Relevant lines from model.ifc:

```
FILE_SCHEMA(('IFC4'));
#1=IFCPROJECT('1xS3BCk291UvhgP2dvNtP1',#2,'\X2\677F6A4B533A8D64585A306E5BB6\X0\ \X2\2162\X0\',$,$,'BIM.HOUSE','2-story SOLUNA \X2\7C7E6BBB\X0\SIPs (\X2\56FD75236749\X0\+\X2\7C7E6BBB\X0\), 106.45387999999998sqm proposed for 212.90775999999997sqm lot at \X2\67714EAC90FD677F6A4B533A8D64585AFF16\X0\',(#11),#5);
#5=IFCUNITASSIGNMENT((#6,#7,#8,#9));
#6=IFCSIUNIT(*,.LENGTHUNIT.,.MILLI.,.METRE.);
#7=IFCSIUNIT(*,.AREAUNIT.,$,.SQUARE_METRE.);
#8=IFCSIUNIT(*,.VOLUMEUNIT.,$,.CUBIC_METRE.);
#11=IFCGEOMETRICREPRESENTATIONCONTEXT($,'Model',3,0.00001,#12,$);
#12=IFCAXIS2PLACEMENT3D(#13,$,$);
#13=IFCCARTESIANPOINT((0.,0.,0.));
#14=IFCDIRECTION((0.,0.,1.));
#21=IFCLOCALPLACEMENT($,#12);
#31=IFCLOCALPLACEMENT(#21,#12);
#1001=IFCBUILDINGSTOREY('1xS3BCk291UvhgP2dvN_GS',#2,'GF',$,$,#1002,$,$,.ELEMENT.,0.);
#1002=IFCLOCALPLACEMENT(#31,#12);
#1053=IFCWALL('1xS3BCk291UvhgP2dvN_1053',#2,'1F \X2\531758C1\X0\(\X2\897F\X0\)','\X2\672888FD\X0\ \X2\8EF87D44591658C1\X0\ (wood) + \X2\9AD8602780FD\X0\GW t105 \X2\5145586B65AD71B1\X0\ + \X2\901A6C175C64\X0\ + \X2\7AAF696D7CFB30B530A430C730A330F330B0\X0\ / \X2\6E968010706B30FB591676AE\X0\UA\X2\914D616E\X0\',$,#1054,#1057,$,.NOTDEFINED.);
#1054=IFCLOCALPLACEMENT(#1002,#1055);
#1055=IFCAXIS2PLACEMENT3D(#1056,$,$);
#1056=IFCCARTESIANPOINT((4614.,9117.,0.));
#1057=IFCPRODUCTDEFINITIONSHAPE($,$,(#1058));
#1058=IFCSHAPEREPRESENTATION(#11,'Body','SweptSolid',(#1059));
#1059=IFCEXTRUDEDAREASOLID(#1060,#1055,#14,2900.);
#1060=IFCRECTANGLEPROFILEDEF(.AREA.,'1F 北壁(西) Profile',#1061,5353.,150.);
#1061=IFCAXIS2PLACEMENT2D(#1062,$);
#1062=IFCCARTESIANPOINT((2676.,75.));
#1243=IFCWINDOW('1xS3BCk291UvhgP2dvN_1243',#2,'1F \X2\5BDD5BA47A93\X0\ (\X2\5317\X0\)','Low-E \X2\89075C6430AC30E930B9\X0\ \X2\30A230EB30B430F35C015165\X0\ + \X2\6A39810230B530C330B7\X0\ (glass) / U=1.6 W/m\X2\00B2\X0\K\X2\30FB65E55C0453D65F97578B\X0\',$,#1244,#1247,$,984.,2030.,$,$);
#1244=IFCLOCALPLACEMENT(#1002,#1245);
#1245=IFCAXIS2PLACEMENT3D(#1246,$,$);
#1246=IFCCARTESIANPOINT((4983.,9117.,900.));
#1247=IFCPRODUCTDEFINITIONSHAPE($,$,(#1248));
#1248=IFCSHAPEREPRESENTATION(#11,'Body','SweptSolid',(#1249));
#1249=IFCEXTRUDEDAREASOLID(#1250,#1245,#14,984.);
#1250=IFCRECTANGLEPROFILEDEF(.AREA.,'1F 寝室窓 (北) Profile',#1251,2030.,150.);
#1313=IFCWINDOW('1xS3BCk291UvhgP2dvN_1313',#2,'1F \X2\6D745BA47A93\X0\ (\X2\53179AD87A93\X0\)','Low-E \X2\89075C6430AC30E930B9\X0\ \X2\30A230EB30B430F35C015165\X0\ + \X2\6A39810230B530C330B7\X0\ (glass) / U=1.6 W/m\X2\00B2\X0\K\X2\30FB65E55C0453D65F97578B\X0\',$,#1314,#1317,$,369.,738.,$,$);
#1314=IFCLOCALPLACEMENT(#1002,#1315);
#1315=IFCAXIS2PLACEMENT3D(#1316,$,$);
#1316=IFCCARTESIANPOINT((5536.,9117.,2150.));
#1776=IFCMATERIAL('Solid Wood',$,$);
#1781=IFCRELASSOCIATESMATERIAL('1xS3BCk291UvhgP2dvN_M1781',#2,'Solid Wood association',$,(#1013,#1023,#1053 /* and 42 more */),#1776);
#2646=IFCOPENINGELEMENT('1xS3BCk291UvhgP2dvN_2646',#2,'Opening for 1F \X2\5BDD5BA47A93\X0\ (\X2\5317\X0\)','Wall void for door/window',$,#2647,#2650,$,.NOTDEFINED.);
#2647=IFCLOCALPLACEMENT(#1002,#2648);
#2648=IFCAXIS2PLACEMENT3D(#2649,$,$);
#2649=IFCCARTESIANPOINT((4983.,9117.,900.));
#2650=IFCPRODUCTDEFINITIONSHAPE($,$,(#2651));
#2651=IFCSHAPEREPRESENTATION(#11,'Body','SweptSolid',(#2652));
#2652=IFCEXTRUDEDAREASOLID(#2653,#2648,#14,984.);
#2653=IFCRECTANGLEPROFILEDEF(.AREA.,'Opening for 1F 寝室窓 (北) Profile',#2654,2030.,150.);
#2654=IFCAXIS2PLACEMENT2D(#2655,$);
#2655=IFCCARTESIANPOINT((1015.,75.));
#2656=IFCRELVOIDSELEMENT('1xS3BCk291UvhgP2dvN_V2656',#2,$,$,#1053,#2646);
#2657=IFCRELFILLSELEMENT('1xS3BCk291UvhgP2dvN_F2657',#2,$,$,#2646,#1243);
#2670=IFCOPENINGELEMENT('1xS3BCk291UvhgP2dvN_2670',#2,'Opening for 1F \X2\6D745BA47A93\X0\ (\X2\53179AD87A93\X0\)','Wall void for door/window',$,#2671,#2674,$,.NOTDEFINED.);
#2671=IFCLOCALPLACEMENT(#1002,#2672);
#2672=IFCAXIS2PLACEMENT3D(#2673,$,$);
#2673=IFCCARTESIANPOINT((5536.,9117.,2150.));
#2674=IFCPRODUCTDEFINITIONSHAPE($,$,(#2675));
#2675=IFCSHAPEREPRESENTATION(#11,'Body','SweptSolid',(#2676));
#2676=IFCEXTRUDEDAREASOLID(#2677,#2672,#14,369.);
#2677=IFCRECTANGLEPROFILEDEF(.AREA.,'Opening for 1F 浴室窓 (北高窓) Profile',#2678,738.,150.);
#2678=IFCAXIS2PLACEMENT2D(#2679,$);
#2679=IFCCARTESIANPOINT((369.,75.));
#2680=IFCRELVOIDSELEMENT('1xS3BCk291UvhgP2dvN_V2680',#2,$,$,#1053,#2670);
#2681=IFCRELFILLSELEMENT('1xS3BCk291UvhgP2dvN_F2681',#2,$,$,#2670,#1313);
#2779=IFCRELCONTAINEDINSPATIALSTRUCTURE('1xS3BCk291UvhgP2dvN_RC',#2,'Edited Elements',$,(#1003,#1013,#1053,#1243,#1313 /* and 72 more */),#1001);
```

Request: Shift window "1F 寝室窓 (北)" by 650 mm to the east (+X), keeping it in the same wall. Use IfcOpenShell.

```python
import ifcopenshell
import ifcopenshell.api.geometry
import ifcopenshell.util.placement
import ifcopenshell.util.unit

model = ifcopenshell.open("model.ifc")
unit_scale = ifcopenshell.util.unit.calculate_unit_scale(model)

window = model.by_guid("1xS3BCk291UvhgP2dvN_1243")
opening = window.FillsVoids[0].RelatingOpeningElement
wall = opening.VoidsElements[0].RelatingBuildingElement

wall_matrix = ifcopenshell.util.placement.get_local_placement(wall.ObjectPlacement)
shift = wall_matrix[:3, 0] * 0.65 / unit_scale
before = ifcopenshell.util.placement.get_local_placement(window.ObjectPlacement)[:3, 3].copy()

# The window is not placed relative to its opening, so move both.
for product in (opening, window):
    matrix = ifcopenshell.util.placement.get_local_placement(product.ObjectPlacement)
    matrix[:3, 3] += shift
    ifcopenshell.api.geometry.edit_object_placement(model, product=product, matrix=matrix, is_si=False)

after = ifcopenshell.util.placement.get_local_placement(window.ObjectPlacement)[:3, 3]
print("window moved by", (after - before).round(3) + 0.0)

model.write("model_edited.ifc")
```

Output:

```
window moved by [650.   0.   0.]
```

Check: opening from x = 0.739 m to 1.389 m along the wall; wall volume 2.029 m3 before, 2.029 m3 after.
